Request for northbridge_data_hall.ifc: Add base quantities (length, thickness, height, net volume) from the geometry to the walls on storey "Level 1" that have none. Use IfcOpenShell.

First a look at what the model holds.

```python
import ifcopenshell
import ifcopenshell.util.element
import ifcopenshell.util.unit

model = ifcopenshell.open("northbridge_data_hall.ifc")
print(model.schema)
for unit_type in ("LENGTHUNIT", "AREAUNIT", "VOLUMEUNIT"):
    print(unit_type, ifcopenshell.util.unit.calculate_unit_scale(model, unit_type))
storey = next(s for s in model.by_type("IfcBuildingStorey") if s.Name == "Level 1")
walls = [e for e in ifcopenshell.util.element.get_decomposition(storey) if e.is_a("IfcWall")]
for e in sorted(walls, key=lambda e: e.id()):
    print(e.id(), e.is_a(), e.Name, list(ifcopenshell.util.element.get_psets(e, qtos_only=True)), sep=" | ")
```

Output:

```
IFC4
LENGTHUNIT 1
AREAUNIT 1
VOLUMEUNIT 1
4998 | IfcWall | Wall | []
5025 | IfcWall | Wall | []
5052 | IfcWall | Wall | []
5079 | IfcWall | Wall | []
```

```python
import ifcopenshell
import ifcopenshell.api.pset
import ifcopenshell.geom
import ifcopenshell.util.element
import ifcopenshell.util.shape
import ifcopenshell.util.unit

model = ifcopenshell.open("northbridge_data_hall.ifc")
unit_scale = ifcopenshell.util.unit.calculate_unit_scale(model)
volume_scale = ifcopenshell.util.unit.calculate_unit_scale(model, "VOLUMEUNIT")
settings = ifcopenshell.geom.settings()

storey = next(s for s in model.by_type("IfcBuildingStorey") if s.Name == "Level 1")
walls = [e for e in ifcopenshell.util.element.get_decomposition(storey) if e.is_a("IfcWall")]

for e in sorted(walls, key=lambda e: e.id()):
    if ifcopenshell.util.element.get_psets(e, qtos_only=True, should_inherit=False):
        continue
    # Geometry comes back in metres, in the element's own axes.
    shape = ifcopenshell.geom.create_shape(settings, e)
    values = {
        "Length": ifcopenshell.util.shape.get_x(shape.geometry) / unit_scale,
        "Width": ifcopenshell.util.shape.get_y(shape.geometry) / unit_scale,
        "Height": ifcopenshell.util.shape.get_z(shape.geometry) / unit_scale,
        "NetVolume": ifcopenshell.util.shape.get_volume(shape.geometry) / volume_scale,
    }
    qto = ifcopenshell.api.pset.add_qto(model, product=e, name="Qto_WallBaseQuantities")
    ifcopenshell.api.pset.edit_qto(model, qto=qto, properties=values)
    print(e.id(), {k: round(v, 3) for k, v in values.items()})

model.write("northbridge_data_hall_v2.ifc")
```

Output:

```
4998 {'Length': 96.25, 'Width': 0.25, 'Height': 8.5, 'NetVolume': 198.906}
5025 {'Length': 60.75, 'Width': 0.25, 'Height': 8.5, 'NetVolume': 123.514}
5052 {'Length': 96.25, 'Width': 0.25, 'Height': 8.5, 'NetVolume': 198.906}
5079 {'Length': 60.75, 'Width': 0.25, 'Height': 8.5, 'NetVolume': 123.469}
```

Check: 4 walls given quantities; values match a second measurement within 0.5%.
